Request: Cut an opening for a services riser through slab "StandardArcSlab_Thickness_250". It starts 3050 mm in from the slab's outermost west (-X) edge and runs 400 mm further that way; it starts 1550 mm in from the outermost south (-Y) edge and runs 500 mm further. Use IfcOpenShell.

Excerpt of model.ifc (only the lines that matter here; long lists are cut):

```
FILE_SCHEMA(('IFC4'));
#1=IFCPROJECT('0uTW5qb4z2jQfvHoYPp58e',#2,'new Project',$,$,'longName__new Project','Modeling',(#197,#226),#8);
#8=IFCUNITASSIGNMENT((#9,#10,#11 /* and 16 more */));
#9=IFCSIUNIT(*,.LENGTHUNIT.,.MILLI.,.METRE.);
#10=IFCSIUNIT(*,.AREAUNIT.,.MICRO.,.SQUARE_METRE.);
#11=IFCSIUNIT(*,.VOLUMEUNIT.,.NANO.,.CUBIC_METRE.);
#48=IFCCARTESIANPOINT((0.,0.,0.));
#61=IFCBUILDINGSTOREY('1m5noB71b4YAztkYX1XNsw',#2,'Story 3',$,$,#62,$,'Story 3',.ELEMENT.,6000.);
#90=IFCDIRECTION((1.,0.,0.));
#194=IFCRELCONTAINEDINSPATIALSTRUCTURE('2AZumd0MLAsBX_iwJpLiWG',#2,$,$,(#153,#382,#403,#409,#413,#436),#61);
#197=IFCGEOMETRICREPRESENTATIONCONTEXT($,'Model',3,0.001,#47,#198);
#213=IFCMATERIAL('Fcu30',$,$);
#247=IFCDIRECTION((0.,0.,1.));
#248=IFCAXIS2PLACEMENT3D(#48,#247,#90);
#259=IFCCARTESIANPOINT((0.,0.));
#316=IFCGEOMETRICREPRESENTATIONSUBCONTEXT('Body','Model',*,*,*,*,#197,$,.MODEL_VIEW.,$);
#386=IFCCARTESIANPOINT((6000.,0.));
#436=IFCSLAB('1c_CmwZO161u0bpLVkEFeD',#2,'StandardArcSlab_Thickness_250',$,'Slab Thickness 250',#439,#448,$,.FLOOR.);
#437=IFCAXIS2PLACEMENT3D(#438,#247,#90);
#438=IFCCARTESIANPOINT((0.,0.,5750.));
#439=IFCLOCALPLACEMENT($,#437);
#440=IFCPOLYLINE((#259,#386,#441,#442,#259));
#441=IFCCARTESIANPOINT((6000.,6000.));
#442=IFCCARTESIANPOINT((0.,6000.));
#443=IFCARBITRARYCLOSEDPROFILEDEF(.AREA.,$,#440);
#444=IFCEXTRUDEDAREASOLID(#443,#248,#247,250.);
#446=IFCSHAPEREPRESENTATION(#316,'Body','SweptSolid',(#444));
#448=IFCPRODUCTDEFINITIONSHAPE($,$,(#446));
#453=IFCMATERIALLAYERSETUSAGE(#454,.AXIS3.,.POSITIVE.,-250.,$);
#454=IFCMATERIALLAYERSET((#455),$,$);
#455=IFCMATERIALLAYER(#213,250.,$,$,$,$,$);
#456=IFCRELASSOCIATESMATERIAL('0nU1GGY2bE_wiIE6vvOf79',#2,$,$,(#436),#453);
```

```python
import numpy as np
import ifcopenshell
import ifcopenshell.api.feature
import ifcopenshell.api.geometry
import ifcopenshell.api.root
import ifcopenshell.geom
import ifcopenshell.util.placement
import ifcopenshell.util.representation
import ifcopenshell.util.shape
import ifcopenshell.util.unit

model = ifcopenshell.open("model.ifc")
unit_scale = ifcopenshell.util.unit.calculate_unit_scale(model)
settings = ifcopenshell.geom.settings()


def volume(element):
    """Net volume in cubic metres, openings subtracted."""
    shape = ifcopenshell.geom.create_shape(settings, element)
    return ifcopenshell.util.shape.get_volume(shape.geometry)


slab = model.by_id(436)
before = volume(slab)

# Extent in the slab's own axes, in metres. The edges named are its -X and -Y sides.
slab_shape = ifcopenshell.geom.create_shape(settings, slab)
vertices = ifcopenshell.util.shape.get_vertices(slab_shape.geometry)
x_min, y_min, bottom = vertices.min(axis=0)
top = vertices[:, 2].max()

opening = ifcopenshell.api.root.create_entity(model, ifc_class="IfcOpeningElement", name="Services riser opening", predefined_type="OPENING")
context = ifcopenshell.util.representation.get_context(model, "Model", "Body", "MODEL_VIEW")
width, depth = 0.4, 0.5
outline = [(0.0, 0.0), (width, 0.0), (width, depth), (0.0, depth), (0.0, 0.0)]
# Overshoot both faces by 50 mm so the cut is clean.
shape = ifcopenshell.api.geometry.add_slab_representation(
    model, context=context, depth=top - bottom + 0.1, polyline=outline
)
ifcopenshell.api.geometry.assign_representation(model, product=opening, representation=shape)

matrix = ifcopenshell.util.placement.get_local_placement(slab.ObjectPlacement)
matrix[:, 3] = matrix @ np.append(np.array([x_min + 3.05, y_min + 1.55, bottom - 0.05]) / unit_scale, 1.0)
ifcopenshell.api.geometry.edit_object_placement(model, product=opening, matrix=matrix, is_si=False)
ifcopenshell.api.feature.add_feature(model, feature=opening, element=slab)

after = volume(slab)

print(f"slab volume {before:.3f} -> {after:.3f} m3")

model.write("model-out.ifc")
```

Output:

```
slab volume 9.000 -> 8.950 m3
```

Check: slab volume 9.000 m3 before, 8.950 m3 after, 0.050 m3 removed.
